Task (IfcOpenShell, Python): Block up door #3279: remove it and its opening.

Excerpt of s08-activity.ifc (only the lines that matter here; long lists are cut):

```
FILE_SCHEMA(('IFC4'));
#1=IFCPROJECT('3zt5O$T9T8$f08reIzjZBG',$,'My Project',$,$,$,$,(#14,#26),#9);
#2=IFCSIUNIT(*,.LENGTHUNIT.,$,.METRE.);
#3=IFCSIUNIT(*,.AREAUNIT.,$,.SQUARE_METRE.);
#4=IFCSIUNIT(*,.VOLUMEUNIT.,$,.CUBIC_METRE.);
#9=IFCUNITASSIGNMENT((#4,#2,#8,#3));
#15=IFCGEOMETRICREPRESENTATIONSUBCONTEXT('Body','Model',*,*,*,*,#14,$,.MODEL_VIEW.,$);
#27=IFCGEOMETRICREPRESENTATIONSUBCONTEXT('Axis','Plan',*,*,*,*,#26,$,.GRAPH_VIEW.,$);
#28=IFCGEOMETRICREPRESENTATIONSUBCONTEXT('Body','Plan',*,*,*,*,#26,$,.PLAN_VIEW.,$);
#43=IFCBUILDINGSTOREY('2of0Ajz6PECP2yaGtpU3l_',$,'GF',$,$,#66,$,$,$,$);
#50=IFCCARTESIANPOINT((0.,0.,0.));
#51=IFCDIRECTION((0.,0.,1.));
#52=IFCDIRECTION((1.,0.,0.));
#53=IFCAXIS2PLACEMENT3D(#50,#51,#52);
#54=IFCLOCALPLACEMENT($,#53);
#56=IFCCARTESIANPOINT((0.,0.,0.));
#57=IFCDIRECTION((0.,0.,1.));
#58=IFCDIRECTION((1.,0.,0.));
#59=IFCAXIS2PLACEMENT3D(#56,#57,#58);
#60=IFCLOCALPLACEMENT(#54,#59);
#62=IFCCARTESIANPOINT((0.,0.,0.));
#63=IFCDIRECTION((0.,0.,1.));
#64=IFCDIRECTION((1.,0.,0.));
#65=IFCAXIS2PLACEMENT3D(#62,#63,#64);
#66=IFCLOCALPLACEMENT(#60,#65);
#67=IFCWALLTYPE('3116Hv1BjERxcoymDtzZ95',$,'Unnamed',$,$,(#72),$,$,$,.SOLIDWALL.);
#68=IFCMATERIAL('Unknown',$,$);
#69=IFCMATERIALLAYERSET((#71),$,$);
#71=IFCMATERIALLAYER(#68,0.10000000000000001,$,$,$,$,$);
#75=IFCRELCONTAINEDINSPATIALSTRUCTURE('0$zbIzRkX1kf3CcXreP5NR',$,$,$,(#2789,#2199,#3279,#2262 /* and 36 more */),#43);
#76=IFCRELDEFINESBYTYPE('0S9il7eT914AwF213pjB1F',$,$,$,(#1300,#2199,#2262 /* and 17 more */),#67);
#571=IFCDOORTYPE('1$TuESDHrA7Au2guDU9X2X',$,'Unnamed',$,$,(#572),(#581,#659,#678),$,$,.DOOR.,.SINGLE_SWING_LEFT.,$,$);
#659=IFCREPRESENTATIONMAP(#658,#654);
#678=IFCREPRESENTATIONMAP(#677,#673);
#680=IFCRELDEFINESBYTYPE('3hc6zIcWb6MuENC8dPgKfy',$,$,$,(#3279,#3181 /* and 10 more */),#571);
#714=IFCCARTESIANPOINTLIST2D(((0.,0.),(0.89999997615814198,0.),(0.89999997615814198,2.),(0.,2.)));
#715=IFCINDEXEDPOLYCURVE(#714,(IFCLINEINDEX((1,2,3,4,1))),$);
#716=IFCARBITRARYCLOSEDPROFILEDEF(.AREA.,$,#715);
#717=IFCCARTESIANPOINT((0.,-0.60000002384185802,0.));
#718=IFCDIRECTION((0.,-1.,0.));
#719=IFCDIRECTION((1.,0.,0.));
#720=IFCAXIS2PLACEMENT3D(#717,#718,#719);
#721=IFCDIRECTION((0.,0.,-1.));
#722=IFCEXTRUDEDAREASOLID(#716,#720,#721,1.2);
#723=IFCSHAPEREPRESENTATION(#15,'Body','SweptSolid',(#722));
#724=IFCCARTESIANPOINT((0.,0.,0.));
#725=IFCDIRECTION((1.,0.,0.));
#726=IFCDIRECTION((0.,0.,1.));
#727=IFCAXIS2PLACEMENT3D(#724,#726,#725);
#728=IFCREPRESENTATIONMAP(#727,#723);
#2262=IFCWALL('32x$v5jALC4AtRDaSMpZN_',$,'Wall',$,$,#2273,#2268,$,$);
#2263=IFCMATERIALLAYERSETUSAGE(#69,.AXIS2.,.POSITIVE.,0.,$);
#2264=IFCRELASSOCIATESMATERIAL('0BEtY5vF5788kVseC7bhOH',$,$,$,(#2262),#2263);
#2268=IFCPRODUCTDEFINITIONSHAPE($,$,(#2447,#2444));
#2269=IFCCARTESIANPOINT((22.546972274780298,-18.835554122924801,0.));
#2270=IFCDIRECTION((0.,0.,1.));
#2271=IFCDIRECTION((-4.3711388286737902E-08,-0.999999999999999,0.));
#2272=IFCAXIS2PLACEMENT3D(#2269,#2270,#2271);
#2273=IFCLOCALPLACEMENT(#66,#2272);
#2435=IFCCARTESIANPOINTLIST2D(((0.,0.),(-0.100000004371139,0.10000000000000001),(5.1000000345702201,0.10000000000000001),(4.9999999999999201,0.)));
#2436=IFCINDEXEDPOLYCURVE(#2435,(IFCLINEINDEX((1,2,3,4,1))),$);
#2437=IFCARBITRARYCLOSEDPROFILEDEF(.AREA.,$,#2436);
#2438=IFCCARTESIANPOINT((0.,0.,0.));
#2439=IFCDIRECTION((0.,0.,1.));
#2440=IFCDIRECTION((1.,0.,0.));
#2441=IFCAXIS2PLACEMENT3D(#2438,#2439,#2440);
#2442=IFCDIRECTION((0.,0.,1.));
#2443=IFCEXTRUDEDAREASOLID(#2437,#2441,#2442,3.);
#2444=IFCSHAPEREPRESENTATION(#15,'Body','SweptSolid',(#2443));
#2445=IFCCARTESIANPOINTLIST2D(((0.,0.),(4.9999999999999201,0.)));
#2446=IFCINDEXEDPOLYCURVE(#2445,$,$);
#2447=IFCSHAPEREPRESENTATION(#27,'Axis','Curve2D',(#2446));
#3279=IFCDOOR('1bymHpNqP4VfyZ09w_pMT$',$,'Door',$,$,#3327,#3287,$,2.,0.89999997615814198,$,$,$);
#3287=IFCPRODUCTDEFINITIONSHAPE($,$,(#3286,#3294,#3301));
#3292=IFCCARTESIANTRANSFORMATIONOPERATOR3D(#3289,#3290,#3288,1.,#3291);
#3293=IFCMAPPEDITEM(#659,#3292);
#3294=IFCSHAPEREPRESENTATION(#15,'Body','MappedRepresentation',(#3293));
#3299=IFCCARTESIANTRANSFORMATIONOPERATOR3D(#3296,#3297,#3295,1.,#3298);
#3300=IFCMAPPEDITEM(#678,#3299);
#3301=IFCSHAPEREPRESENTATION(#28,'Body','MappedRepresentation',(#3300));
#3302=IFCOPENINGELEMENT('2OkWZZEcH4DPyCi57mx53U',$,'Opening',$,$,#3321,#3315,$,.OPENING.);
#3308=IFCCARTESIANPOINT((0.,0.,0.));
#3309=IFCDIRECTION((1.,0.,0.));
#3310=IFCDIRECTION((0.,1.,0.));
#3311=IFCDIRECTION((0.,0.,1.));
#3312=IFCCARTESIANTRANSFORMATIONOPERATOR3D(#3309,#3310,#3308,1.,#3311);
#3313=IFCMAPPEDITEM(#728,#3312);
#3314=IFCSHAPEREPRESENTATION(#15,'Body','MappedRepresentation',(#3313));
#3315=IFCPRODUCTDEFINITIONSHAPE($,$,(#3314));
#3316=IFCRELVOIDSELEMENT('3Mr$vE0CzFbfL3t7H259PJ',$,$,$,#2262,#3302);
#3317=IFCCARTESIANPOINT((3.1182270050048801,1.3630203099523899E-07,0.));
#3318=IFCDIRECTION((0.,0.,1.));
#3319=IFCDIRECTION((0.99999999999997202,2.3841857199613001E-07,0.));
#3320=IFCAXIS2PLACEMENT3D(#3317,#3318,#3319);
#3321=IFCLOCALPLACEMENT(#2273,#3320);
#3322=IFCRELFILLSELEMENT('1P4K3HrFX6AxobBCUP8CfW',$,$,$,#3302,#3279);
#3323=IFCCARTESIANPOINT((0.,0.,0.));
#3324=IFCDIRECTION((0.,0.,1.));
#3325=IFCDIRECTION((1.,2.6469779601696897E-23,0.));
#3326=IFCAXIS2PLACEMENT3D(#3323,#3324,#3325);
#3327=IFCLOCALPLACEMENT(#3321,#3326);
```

```python
import ifcopenshell
import ifcopenshell.api.feature
import ifcopenshell.api.root
import ifcopenshell.geom
import ifcopenshell.util.shape

model = ifcopenshell.open("s08-activity.ifc")
settings = ifcopenshell.geom.settings()


def volume(element):
    """Net volume in cubic metres, openings subtracted."""
    shape = ifcopenshell.geom.create_shape(settings, element)
    return ifcopenshell.util.shape.get_volume(shape.geometry)


door = model.by_id(3279)
opening = door.FillsVoids[0].RelatingOpeningElement
wall = opening.VoidsElements[0].RelatingBuildingElement
before = volume(wall)

ifcopenshell.api.root.remove_product(model, product=door)
ifcopenshell.api.feature.remove_feature(model, feature=opening)

after = volume(wall)

print(f"wall volume {before:.3f} -> {after:.3f} m3")

model.write("s08-activity-out.ifc")
```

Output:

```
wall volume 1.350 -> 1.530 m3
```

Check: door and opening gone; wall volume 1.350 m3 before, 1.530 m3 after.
